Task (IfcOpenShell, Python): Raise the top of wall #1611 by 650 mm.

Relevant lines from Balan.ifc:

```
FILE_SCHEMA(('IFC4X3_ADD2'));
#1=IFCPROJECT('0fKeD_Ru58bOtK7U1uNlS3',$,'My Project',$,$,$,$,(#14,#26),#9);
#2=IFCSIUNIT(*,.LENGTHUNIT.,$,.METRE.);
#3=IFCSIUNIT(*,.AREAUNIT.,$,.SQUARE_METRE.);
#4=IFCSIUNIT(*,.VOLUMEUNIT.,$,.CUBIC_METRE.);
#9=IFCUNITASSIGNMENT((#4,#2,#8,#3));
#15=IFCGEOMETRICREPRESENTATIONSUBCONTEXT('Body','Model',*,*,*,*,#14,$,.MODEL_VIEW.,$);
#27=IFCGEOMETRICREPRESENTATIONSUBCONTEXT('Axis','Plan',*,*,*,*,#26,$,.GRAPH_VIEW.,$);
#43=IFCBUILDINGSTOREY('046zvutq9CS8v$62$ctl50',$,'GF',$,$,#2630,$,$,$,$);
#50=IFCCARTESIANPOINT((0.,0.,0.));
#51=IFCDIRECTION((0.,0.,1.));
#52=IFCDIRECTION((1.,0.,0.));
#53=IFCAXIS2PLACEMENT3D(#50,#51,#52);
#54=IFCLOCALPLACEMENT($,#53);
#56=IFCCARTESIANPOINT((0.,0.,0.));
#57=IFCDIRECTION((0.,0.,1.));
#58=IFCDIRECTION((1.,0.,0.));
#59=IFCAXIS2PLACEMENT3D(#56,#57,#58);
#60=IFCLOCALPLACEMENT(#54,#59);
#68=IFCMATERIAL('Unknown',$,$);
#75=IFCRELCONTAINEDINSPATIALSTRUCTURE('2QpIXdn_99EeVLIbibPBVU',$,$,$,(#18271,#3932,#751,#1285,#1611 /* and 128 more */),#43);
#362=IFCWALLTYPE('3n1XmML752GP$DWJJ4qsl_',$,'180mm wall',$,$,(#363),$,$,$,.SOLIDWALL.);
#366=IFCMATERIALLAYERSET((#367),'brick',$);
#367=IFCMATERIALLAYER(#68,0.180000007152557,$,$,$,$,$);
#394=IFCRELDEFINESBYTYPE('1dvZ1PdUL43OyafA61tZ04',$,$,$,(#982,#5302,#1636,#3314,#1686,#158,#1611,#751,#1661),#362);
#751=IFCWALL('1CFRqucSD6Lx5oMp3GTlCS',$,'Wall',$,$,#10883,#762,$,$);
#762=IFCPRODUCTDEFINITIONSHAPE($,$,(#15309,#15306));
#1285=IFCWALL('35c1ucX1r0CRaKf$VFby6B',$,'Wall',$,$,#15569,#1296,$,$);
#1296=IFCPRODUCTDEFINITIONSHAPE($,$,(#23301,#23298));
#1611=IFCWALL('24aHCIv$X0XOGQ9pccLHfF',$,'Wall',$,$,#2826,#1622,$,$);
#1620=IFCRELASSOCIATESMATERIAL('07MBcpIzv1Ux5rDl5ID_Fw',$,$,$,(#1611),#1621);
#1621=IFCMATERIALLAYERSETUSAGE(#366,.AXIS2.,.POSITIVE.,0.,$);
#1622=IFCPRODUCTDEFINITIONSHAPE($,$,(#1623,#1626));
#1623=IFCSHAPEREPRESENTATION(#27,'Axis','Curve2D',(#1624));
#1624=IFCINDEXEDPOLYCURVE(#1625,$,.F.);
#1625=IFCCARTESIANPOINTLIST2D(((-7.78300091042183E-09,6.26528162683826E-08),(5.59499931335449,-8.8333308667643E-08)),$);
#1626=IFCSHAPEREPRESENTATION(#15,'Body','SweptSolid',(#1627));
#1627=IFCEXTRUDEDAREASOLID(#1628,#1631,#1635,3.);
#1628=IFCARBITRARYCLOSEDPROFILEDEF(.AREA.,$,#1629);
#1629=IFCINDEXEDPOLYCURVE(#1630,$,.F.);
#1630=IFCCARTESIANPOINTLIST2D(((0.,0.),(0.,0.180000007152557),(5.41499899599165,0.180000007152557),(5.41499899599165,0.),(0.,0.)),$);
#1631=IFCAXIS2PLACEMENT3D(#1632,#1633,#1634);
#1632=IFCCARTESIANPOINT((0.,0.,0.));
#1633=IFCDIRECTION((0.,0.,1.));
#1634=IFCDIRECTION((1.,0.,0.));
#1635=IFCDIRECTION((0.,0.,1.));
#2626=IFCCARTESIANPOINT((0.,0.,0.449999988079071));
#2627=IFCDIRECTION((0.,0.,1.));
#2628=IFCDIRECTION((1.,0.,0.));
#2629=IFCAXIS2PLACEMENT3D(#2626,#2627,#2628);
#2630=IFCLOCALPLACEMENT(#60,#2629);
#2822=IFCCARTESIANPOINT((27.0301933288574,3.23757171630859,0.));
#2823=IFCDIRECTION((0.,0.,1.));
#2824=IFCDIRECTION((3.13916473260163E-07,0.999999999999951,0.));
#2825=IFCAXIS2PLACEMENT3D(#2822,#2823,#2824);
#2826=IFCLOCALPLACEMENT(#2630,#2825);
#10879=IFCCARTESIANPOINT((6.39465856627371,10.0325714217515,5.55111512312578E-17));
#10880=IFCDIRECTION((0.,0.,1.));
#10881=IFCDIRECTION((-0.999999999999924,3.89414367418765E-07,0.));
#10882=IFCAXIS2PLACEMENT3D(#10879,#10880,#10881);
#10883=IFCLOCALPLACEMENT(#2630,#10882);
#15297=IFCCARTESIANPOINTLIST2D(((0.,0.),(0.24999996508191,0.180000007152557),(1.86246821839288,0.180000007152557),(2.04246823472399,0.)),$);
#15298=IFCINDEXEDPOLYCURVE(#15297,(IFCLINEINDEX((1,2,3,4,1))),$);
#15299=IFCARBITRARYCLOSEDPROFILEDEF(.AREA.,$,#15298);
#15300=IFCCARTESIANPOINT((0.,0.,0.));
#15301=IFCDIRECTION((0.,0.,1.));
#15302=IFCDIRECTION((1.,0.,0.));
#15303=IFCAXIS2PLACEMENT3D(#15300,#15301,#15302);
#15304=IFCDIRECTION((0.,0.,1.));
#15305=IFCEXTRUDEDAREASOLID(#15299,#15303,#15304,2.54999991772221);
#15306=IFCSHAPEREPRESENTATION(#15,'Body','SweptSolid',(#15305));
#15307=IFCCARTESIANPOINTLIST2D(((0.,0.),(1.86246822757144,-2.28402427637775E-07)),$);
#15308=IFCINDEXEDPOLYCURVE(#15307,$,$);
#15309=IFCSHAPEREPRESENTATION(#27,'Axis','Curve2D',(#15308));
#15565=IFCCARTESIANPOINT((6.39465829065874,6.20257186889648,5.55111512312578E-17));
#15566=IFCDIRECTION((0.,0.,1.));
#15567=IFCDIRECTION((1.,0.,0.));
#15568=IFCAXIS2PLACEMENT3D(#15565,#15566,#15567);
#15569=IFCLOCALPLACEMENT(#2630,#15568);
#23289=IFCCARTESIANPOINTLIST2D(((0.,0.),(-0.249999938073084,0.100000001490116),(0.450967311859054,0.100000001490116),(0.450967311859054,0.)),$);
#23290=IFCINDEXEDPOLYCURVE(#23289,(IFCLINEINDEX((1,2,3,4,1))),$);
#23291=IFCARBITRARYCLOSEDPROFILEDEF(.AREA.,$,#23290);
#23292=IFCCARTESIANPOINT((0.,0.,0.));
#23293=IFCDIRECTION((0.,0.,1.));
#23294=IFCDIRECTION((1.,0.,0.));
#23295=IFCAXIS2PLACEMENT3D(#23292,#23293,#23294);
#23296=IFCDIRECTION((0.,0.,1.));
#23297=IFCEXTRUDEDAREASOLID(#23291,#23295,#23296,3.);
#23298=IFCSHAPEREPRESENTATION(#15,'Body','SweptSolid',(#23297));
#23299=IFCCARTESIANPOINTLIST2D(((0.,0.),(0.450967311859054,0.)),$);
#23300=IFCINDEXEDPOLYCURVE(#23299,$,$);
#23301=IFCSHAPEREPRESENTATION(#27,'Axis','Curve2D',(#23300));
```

```python
import ifcopenshell
import ifcopenshell.geom
import ifcopenshell.util.representation
import ifcopenshell.util.shape

model = ifcopenshell.open("Balan.ifc")
settings = ifcopenshell.geom.settings()


def volume(element):
    """Net volume in cubic metres, openings subtracted."""
    shape = ifcopenshell.geom.create_shape(settings, element)
    return ifcopenshell.util.shape.get_volume(shape.geometry)


wall = model.by_id(1611)
before = volume(wall)

body = ifcopenshell.util.representation.get_representation(wall, "Model", "Body")
solid = body.Items[0]
old_height = solid.Depth
solid.Depth += 0.65
after = volume(wall)

print(f"height {old_height:g} -> {solid.Depth:g}, volume {before:.3f} -> {after:.3f} m3")

model.write("Balan_updated.ifc")
```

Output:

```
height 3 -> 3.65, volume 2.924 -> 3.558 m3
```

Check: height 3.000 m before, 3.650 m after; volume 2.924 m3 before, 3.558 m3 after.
